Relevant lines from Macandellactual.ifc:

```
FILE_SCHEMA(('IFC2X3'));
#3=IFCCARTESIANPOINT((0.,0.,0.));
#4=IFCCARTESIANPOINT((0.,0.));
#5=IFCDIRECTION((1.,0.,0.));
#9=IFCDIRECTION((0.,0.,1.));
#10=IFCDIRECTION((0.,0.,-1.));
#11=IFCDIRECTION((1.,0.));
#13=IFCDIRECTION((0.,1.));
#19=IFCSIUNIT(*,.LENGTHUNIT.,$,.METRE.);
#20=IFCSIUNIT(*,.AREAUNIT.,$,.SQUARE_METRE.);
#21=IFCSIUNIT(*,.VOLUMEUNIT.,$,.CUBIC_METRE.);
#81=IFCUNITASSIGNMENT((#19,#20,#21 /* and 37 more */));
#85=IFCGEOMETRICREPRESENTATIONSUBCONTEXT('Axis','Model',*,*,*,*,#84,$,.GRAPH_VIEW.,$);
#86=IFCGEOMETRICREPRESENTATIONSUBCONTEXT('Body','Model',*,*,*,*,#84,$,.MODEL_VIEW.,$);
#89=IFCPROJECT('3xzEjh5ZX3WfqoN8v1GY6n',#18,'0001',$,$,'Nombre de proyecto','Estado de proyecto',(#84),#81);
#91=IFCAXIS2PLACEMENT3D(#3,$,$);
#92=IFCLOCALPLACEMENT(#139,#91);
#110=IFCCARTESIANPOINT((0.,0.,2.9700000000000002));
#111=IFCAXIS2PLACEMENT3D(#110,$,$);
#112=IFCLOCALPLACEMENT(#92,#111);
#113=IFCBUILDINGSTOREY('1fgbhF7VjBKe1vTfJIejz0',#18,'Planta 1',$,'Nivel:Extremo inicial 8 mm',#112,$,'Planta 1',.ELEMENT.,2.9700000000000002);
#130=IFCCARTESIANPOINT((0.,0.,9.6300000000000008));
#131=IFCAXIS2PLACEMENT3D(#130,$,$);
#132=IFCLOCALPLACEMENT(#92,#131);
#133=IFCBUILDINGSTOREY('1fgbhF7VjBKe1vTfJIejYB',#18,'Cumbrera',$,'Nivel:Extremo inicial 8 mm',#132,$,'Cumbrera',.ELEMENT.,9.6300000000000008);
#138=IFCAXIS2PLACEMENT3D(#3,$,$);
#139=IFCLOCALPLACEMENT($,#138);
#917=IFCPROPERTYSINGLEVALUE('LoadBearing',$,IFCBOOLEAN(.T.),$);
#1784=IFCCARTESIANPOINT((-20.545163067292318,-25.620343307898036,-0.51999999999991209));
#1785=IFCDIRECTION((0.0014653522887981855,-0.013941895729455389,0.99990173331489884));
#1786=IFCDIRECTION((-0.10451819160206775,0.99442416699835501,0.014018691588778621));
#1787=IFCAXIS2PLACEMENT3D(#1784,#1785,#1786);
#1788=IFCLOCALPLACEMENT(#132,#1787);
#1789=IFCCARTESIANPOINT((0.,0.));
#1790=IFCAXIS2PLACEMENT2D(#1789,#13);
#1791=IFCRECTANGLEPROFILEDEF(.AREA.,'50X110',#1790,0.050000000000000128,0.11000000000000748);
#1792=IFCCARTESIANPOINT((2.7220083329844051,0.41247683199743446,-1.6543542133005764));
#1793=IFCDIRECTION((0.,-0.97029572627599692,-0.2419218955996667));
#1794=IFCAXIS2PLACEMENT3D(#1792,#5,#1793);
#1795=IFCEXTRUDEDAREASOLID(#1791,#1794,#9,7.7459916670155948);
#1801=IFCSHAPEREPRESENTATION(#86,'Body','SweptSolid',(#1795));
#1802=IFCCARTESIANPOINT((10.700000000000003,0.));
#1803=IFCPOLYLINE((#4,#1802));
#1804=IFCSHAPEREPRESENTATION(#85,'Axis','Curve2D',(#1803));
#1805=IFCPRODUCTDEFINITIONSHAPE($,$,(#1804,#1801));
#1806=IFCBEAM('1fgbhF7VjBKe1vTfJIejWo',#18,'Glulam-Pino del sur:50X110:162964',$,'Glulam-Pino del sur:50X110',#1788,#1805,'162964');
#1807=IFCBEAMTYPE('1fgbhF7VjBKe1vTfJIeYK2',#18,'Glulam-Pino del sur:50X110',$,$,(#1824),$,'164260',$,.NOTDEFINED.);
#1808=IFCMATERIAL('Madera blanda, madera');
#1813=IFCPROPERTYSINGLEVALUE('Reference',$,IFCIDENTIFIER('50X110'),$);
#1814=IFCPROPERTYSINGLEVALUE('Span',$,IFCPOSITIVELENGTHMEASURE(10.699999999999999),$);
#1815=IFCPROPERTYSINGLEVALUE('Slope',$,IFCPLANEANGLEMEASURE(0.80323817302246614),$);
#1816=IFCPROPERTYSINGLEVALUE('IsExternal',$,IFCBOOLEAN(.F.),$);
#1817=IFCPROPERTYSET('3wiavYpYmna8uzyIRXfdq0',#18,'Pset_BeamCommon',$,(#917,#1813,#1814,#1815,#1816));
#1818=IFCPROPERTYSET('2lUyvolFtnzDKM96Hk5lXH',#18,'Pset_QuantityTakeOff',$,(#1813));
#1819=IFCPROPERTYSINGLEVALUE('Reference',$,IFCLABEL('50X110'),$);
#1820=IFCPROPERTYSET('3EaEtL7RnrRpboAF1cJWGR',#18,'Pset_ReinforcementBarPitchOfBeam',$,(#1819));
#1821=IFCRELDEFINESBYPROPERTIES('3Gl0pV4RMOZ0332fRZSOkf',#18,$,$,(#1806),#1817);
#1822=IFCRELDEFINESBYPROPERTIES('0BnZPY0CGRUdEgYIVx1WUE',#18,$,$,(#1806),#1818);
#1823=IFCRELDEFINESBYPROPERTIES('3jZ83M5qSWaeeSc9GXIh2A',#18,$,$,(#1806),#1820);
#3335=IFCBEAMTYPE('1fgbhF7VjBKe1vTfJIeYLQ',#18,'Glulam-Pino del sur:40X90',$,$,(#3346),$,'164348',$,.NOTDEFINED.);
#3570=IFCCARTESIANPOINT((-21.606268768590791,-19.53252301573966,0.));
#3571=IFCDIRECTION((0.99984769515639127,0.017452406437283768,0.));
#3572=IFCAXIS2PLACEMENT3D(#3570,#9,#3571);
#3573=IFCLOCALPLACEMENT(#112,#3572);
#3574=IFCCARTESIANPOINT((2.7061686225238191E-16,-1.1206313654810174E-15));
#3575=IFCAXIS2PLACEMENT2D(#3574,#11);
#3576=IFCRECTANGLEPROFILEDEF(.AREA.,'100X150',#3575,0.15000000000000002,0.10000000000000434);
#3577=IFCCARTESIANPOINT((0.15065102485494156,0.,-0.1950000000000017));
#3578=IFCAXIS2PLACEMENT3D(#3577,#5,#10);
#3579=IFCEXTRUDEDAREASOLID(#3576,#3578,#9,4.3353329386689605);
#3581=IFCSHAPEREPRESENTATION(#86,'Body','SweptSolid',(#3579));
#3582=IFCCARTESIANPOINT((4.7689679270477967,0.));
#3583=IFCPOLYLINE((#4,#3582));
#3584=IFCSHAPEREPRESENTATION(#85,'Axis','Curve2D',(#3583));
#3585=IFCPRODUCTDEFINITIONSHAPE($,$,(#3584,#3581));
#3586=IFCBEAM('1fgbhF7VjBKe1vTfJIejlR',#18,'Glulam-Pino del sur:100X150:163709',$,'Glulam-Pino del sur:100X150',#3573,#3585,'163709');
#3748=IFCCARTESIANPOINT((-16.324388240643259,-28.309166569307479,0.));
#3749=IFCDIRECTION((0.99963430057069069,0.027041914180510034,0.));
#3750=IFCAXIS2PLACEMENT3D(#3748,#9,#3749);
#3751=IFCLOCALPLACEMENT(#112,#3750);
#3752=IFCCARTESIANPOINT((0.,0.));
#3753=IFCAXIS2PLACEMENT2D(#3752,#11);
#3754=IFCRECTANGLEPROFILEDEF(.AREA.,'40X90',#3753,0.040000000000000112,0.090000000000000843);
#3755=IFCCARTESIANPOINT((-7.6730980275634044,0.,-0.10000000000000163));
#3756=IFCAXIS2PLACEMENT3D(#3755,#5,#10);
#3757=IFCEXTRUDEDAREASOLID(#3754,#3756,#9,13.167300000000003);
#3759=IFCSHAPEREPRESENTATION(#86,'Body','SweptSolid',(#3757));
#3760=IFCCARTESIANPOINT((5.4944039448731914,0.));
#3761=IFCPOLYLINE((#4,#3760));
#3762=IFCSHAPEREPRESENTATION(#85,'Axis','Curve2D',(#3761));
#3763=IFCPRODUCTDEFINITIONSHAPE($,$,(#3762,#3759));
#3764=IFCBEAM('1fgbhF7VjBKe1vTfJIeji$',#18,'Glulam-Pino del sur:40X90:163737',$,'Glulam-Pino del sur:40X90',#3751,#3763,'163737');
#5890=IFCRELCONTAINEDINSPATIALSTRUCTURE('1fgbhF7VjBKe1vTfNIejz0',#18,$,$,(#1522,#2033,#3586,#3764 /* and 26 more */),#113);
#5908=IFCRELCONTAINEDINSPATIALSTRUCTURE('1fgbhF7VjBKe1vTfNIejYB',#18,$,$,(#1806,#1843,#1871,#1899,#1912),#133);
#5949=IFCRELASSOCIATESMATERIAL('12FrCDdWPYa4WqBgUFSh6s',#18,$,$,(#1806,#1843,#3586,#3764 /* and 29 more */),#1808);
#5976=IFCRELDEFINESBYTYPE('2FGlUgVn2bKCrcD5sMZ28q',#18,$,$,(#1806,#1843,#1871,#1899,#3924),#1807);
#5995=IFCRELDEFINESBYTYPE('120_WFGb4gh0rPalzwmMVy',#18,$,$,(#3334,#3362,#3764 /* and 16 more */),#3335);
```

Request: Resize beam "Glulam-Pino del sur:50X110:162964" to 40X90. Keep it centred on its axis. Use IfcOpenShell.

```python
import ifcopenshell
import ifcopenshell.api.pset
import ifcopenshell.api.type
import ifcopenshell.util.element
import ifcopenshell.util.representation

model = ifcopenshell.open("Macandellactual.ifc")

member = model.by_guid("1fgbhF7VjBKe1vTfJIejWo")
source = next(p for p in model.by_type("IfcRectangleProfileDef") if p.ProfileName == "40X90")

body = ifcopenshell.util.representation.get_representation(member, "Model", "Body")
solid = body.Items[0]
old_profile = solid.SweptArea

# Copy the section's sizes but keep this member's own profile position.
profile = ifcopenshell.util.element.copy(model, source)
profile.Position = old_profile.Position
solid.SweptArea = profile
if not model.get_total_inverses(old_profile):
    ifcopenshell.util.element.remove_deep2(model, old_profile)

new_type = model.by_guid("1fgbhF7VjBKe1vTfJIeYLQ")
ifcopenshell.api.type.assign_type(
    model, related_objects=[member], relating_type=new_type, should_map_representations=False
)
member.Name = member.Name.replace("50X110", "40X90")
member.ObjectType = "Glulam-Pino del sur:40X90"
pset = model.by_id(ifcopenshell.util.element.get_pset(member, "Pset_BeamCommon", should_inherit=False)["id"])
ifcopenshell.api.pset.edit_pset(model, pset=pset, properties={"Reference": "40X90"})
pset = model.by_id(ifcopenshell.util.element.get_pset(member, "Pset_QuantityTakeOff", should_inherit=False)["id"])
ifcopenshell.api.pset.edit_pset(model, pset=pset, properties={"Reference": "40X90"})
pset = model.by_id(ifcopenshell.util.element.get_pset(member, "Pset_ReinforcementBarPitchOfBeam", should_inherit=False)["id"])
ifcopenshell.api.pset.edit_pset(model, pset=pset, properties={"Reference": "40X90"})

print(solid.SweptArea)

model.write("Macandellactual_rev.ifc")
```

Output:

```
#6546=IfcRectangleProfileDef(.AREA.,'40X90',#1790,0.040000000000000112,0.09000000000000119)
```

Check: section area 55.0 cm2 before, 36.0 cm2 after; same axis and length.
